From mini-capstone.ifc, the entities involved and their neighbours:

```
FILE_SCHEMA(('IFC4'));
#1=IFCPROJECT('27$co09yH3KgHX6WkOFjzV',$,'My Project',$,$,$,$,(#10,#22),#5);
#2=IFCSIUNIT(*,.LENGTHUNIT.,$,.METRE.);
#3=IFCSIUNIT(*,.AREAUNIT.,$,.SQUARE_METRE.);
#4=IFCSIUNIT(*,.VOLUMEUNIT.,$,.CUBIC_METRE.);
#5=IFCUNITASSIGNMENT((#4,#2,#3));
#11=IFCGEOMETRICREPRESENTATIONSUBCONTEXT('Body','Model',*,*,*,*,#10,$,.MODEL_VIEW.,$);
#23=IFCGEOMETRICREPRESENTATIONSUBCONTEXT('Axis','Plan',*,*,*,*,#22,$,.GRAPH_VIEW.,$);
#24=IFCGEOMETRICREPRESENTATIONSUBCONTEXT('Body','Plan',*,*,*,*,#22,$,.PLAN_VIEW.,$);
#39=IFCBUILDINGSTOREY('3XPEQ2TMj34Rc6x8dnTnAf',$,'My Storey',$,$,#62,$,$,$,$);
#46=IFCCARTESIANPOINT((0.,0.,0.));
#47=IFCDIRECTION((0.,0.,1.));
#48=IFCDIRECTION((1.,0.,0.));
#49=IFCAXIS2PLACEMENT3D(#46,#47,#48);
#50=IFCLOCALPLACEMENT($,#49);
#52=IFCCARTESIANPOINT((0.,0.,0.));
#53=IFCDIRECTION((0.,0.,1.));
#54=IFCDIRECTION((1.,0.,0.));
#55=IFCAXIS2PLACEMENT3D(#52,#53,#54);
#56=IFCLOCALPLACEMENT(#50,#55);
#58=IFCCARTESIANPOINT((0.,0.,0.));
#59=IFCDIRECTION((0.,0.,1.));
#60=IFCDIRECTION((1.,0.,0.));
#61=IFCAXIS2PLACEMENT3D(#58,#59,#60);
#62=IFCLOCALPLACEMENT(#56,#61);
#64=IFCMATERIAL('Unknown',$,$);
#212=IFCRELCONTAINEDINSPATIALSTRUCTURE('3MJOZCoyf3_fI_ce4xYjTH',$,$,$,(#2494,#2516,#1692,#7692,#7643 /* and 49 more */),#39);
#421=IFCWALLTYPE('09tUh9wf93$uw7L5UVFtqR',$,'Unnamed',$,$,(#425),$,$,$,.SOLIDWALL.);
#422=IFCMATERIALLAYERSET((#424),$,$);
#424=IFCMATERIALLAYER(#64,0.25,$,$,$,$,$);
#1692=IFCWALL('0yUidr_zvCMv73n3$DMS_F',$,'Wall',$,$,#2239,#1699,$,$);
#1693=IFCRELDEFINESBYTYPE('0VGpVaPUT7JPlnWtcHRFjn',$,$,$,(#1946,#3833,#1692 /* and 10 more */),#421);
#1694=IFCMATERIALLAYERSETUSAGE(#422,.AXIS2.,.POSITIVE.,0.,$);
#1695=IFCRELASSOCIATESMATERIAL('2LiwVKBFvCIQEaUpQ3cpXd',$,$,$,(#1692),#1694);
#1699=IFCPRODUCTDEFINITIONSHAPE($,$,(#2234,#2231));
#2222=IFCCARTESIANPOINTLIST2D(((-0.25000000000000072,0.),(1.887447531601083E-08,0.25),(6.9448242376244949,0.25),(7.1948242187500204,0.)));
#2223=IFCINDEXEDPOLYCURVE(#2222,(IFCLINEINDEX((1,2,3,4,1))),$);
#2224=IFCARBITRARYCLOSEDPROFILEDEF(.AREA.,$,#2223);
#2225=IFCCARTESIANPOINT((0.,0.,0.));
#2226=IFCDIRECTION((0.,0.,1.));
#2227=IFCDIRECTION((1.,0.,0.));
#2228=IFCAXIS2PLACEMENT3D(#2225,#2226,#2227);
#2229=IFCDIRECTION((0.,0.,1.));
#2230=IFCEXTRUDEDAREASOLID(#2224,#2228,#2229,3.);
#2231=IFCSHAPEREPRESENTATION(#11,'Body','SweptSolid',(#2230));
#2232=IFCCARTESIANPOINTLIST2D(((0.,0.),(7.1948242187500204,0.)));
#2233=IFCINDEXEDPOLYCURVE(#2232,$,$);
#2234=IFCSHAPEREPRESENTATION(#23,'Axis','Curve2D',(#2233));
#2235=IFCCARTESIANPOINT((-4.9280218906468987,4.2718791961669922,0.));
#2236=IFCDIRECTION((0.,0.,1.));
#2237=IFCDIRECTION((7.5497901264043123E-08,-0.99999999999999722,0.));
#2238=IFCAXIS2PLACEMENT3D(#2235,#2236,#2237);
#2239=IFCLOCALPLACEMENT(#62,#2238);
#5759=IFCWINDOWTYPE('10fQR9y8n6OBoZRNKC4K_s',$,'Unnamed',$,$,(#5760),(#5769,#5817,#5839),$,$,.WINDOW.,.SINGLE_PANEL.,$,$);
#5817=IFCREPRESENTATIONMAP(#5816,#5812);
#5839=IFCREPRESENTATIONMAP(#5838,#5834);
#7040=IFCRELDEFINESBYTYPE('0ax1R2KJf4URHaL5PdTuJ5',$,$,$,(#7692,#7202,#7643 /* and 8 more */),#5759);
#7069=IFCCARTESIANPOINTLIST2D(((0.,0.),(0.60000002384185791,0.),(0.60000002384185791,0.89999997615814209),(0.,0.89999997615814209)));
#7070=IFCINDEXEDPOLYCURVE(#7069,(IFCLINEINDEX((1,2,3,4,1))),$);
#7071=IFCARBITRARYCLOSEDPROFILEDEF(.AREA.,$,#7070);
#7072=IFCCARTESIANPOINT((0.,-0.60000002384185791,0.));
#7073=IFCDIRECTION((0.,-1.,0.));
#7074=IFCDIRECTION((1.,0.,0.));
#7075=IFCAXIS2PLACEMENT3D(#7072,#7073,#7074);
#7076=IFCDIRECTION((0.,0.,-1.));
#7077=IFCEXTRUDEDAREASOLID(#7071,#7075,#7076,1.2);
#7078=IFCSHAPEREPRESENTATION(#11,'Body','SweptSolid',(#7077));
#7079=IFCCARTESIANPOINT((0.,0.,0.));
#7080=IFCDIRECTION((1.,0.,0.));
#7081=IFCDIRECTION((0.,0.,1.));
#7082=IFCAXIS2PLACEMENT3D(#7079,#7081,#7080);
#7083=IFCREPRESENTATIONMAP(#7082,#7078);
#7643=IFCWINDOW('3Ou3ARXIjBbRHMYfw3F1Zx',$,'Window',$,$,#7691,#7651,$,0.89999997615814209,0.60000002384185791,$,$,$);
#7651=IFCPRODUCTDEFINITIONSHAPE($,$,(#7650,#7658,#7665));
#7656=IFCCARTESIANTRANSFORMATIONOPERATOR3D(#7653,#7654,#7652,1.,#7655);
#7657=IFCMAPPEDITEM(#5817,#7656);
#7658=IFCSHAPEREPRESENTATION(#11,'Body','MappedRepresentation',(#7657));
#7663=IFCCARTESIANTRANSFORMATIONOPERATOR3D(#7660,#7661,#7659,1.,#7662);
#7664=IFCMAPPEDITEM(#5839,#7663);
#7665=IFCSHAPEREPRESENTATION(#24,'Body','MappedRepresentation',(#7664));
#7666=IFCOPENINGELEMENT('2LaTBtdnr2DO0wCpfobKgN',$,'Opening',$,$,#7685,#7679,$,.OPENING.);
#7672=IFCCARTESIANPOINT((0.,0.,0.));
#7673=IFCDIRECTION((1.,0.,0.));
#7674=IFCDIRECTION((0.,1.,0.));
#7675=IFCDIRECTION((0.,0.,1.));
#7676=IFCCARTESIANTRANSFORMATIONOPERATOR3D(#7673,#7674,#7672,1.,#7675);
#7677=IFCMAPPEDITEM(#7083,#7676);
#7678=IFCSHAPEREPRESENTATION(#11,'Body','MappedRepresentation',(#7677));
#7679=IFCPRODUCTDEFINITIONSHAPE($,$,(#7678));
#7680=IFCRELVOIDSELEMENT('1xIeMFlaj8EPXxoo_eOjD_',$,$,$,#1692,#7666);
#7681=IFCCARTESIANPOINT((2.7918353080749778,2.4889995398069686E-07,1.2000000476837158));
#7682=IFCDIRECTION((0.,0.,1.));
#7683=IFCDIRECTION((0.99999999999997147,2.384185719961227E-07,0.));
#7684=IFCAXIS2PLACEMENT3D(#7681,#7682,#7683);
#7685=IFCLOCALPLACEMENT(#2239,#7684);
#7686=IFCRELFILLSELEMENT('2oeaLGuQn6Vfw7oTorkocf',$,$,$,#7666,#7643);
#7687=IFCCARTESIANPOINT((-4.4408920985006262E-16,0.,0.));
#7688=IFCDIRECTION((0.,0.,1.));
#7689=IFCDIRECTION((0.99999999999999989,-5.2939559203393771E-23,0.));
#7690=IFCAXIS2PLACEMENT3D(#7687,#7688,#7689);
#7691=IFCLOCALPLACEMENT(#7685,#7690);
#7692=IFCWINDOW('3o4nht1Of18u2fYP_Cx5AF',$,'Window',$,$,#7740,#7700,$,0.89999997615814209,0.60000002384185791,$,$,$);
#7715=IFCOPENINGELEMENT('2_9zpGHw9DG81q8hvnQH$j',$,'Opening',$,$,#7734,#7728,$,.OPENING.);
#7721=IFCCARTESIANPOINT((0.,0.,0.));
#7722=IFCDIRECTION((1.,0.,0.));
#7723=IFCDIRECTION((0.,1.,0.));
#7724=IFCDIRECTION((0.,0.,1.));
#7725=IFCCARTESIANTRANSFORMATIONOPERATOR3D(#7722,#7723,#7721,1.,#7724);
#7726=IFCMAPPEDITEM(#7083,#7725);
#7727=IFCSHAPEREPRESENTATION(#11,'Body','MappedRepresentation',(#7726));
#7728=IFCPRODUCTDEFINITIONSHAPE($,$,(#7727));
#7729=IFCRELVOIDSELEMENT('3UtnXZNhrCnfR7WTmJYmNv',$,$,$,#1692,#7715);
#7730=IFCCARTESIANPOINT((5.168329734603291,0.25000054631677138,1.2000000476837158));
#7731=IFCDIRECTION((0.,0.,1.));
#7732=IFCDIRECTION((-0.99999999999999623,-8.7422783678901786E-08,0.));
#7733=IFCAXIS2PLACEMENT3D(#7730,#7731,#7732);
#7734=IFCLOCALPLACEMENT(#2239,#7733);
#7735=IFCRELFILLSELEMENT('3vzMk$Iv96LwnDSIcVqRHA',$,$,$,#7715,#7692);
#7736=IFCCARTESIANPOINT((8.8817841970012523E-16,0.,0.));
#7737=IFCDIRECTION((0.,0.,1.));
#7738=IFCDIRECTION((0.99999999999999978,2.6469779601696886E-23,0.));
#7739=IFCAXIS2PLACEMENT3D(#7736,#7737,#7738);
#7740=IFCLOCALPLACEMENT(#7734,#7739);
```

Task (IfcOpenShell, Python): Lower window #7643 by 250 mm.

```python
import numpy as np
import ifcopenshell
import ifcopenshell.api.geometry
import ifcopenshell.util.placement
import ifcopenshell.util.unit

model = ifcopenshell.open("mini-capstone.ifc")
unit_scale = ifcopenshell.util.unit.calculate_unit_scale(model)

window = model.by_guid("3Ou3ARXIjBbRHMYfw3F1Zx")
opening = window.FillsVoids[0].RelatingOpeningElement
dz = -0.25 / unit_scale

shift = np.array([0.0, 0.0, dz])
# The window is placed relative to its opening, so it follows when the opening moves.
matrix = ifcopenshell.util.placement.get_local_placement(opening.ObjectPlacement)
matrix[:3, 3] += shift
ifcopenshell.api.geometry.edit_object_placement(
    model, product=opening, matrix=matrix, is_si=False, should_transform_children=True
)

print(f"moved by {dz * unit_scale:+.3f} m")

model.write("mini-capstone_edited.ifc")
```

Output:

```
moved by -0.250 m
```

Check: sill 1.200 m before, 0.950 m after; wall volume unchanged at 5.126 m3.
